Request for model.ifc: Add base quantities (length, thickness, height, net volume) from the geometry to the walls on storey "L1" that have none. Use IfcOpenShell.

First a look at what the model holds.

```python
import ifcopenshell
import ifcopenshell.util.element
import ifcopenshell.util.unit

model = ifcopenshell.open("model.ifc")
print(model.schema)
for unit_type in ("LENGTHUNIT", "AREAUNIT", "VOLUMEUNIT"):
    print(unit_type, ifcopenshell.util.unit.calculate_unit_scale(model, unit_type))
storey = next(s for s in model.by_type("IfcBuildingStorey") if s.Name == "L1")
walls = [e for e in ifcopenshell.util.element.get_decomposition(storey) if e.is_a("IfcWall")]
for e in sorted(walls, key=lambda e: e.id()):
    print(e.id(), e.is_a(), e.Name, list(ifcopenshell.util.element.get_psets(e, qtos_only=True)), sep=" | ")
```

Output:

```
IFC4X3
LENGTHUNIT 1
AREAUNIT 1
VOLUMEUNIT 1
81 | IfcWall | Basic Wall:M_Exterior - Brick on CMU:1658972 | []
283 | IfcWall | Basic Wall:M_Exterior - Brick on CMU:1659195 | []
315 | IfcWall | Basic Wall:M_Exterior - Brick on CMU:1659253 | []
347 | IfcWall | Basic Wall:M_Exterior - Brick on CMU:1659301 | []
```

```python
import ifcopenshell
import ifcopenshell.api.pset
import ifcopenshell.geom
import ifcopenshell.util.element
import ifcopenshell.util.shape
import ifcopenshell.util.unit

model = ifcopenshell.open("model.ifc")
unit_scale = ifcopenshell.util.unit.calculate_unit_scale(model)
volume_scale = ifcopenshell.util.unit.calculate_unit_scale(model, "VOLUMEUNIT")
settings = ifcopenshell.geom.settings()

storey = next(s for s in model.by_type("IfcBuildingStorey") if s.Name == "L1")
walls = [e for e in ifcopenshell.util.element.get_decomposition(storey) if e.is_a("IfcWall")]

for e in sorted(walls, key=lambda e: e.id()):
    if ifcopenshell.util.element.get_psets(e, qtos_only=True, should_inherit=False):
        continue
    # Geometry comes back in metres, in the element's own axes.
    shape = ifcopenshell.geom.create_shape(settings, e)
    values = {
        "Length": ifcopenshell.util.shape.get_x(shape.geometry) / unit_scale,
        "Width": ifcopenshell.util.shape.get_y(shape.geometry) / unit_scale,
        "Height": ifcopenshell.util.shape.get_z(shape.geometry) / unit_scale,
        "NetVolume": ifcopenshell.util.shape.get_volume(shape.geometry) / volume_scale,
    }
    qto = ifcopenshell.api.pset.add_qto(model, product=e, name="Qto_WallBaseQuantities")
    ifcopenshell.api.pset.edit_qto(model, qto=qto, properties=values)
    print(e.id(), {k: round(v, 3) for k, v in values.items()})

model.write("model_edited.ifc")
```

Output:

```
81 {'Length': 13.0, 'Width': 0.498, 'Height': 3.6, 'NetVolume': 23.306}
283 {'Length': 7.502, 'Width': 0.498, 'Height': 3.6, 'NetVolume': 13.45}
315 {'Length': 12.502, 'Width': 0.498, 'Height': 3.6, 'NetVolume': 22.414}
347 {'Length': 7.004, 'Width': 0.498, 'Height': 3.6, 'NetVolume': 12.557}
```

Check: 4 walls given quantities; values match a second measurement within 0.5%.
